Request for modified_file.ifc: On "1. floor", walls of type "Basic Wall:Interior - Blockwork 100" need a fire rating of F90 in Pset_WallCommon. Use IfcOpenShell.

First a look at what the model holds.

```python
import ifcopenshell
import ifcopenshell.util.element

model = ifcopenshell.open("modified_file.ifc")
print(model.schema)
storey = next(s for s in model.by_type("IfcBuildingStorey") if s.Name == "1. floor")
walls = [e for e in ifcopenshell.util.element.get_decomposition(storey) if e.is_a("IfcWall")]
seen = {}
for e in walls:
    element_type = ifcopenshell.util.element.get_type(e)
    key = (element_type.Name if element_type != e and element_type else None, ifcopenshell.util.element.get_pset(e, "Pset_WallCommon", "FireRating"))
    seen[key] = seen.get(key, 0) + 1
for (name, value), count in sorted(seen.items(), key=str):
    print(count, "x", name, "|", value)
```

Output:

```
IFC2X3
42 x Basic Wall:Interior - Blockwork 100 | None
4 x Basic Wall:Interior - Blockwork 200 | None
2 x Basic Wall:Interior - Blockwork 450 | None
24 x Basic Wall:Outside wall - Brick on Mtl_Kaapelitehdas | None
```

```python
import ifcopenshell
import ifcopenshell.api.pset
import ifcopenshell.util.element

model = ifcopenshell.open("modified_file.ifc")

storey = next(s for s in model.by_type("IfcBuildingStorey") if s.Name == "1. floor")
walls = [e for e in ifcopenshell.util.element.get_decomposition(storey) if e.is_a("IfcWall")]

count = 0
for e in walls:
    element_type = ifcopenshell.util.element.get_type(e)
    if element_type in (None, e) or element_type.Name != "Basic Wall:Interior - Blockwork 100":
        continue
    # add_pset returns the element's existing set when there is one.
    pset = ifcopenshell.api.pset.add_pset(model, product=e, name="Pset_WallCommon")
    ifcopenshell.api.pset.edit_pset(model, pset=pset, properties={"FireRating": "F90"})
    count += 1

print(count, "walls updated")

model.write("modified_file-out.ifc")
```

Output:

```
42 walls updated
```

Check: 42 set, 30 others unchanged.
